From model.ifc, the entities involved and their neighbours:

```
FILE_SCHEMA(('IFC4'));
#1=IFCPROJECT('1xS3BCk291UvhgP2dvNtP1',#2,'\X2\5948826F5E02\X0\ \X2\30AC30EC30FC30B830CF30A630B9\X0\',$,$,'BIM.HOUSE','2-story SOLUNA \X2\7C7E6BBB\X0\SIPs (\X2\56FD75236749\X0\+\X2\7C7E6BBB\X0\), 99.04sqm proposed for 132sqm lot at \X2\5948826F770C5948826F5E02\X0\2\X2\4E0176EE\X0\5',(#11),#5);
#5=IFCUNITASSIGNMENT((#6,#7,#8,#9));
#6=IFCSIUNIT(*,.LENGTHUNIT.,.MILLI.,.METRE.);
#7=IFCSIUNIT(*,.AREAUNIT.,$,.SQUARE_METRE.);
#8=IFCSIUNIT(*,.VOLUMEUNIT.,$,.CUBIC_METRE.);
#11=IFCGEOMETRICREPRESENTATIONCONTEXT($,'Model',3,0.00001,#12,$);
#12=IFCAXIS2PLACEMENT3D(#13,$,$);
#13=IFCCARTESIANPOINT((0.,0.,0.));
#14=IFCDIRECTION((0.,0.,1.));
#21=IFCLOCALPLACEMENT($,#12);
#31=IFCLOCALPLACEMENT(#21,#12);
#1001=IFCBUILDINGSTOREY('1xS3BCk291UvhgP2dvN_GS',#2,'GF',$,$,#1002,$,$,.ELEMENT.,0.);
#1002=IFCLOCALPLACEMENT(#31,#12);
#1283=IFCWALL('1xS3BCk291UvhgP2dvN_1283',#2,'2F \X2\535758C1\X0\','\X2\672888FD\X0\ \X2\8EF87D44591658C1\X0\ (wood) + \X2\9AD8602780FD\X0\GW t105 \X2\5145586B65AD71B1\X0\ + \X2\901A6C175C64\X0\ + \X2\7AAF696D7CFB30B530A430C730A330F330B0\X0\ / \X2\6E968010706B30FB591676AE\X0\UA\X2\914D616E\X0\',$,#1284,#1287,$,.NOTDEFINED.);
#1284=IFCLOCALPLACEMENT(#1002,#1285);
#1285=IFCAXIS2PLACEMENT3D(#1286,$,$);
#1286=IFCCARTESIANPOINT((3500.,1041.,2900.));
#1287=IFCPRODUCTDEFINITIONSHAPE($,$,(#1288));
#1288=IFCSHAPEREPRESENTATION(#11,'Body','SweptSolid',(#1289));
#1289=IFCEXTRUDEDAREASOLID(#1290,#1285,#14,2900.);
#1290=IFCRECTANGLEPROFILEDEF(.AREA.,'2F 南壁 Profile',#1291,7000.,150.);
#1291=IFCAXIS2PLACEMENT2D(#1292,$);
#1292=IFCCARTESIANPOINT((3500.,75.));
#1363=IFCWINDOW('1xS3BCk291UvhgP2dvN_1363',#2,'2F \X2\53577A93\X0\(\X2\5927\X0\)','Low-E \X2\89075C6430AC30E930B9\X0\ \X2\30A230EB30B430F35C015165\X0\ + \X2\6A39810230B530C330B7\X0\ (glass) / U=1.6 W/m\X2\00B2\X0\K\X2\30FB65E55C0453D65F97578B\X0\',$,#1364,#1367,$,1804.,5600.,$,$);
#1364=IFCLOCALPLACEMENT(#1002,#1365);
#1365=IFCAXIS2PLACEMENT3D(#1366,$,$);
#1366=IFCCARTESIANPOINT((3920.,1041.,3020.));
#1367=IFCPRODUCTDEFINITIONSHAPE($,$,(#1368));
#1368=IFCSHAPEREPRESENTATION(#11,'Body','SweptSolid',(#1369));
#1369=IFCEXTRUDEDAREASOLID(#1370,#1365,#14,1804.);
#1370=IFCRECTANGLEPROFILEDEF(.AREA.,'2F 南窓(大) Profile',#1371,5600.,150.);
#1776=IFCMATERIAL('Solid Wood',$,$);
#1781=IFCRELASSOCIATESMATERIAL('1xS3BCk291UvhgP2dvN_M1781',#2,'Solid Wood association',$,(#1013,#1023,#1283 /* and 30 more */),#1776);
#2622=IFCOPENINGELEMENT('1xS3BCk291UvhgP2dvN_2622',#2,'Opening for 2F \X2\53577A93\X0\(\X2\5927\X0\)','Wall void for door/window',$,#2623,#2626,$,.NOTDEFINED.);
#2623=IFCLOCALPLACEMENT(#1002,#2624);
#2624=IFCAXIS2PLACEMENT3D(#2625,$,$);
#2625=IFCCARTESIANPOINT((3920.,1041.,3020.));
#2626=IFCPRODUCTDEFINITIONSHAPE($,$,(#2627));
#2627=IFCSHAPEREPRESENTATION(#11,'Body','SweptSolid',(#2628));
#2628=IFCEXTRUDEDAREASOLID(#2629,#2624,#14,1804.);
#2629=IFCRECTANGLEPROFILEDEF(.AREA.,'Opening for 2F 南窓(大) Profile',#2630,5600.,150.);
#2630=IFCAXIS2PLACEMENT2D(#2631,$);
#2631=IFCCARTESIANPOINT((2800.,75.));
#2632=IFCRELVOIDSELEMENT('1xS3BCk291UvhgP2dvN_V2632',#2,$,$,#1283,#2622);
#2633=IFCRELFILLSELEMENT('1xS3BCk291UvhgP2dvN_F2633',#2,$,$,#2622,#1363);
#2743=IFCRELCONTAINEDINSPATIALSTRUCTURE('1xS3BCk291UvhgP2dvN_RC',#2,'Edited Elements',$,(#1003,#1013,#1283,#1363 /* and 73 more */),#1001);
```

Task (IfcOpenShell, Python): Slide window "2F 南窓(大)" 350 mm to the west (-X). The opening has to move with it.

```python
import ifcopenshell
import ifcopenshell.api.geometry
import ifcopenshell.util.placement
import ifcopenshell.util.unit

model = ifcopenshell.open("model.ifc")
unit_scale = ifcopenshell.util.unit.calculate_unit_scale(model)

window = model.by_guid("1xS3BCk291UvhgP2dvN_1363")
opening = window.FillsVoids[0].RelatingOpeningElement
wall = opening.VoidsElements[0].RelatingBuildingElement

wall_matrix = ifcopenshell.util.placement.get_local_placement(wall.ObjectPlacement)
shift = wall_matrix[:3, 0] * -0.35 / unit_scale
before = ifcopenshell.util.placement.get_local_placement(window.ObjectPlacement)[:3, 3].copy()

# The window is not placed relative to its opening, so move both.
for product in (opening, window):
    matrix = ifcopenshell.util.placement.get_local_placement(product.ObjectPlacement)
    matrix[:3, 3] += shift
    ifcopenshell.api.geometry.edit_object_placement(model, product=product, matrix=matrix, is_si=False)

after = ifcopenshell.util.placement.get_local_placement(window.ObjectPlacement)[:3, 3]
print("window moved by", (after - before).round(3) + 0.0)

model.write("model_updated.ifc")
```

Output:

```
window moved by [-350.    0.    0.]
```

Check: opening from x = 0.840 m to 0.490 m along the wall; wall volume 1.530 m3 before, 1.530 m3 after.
